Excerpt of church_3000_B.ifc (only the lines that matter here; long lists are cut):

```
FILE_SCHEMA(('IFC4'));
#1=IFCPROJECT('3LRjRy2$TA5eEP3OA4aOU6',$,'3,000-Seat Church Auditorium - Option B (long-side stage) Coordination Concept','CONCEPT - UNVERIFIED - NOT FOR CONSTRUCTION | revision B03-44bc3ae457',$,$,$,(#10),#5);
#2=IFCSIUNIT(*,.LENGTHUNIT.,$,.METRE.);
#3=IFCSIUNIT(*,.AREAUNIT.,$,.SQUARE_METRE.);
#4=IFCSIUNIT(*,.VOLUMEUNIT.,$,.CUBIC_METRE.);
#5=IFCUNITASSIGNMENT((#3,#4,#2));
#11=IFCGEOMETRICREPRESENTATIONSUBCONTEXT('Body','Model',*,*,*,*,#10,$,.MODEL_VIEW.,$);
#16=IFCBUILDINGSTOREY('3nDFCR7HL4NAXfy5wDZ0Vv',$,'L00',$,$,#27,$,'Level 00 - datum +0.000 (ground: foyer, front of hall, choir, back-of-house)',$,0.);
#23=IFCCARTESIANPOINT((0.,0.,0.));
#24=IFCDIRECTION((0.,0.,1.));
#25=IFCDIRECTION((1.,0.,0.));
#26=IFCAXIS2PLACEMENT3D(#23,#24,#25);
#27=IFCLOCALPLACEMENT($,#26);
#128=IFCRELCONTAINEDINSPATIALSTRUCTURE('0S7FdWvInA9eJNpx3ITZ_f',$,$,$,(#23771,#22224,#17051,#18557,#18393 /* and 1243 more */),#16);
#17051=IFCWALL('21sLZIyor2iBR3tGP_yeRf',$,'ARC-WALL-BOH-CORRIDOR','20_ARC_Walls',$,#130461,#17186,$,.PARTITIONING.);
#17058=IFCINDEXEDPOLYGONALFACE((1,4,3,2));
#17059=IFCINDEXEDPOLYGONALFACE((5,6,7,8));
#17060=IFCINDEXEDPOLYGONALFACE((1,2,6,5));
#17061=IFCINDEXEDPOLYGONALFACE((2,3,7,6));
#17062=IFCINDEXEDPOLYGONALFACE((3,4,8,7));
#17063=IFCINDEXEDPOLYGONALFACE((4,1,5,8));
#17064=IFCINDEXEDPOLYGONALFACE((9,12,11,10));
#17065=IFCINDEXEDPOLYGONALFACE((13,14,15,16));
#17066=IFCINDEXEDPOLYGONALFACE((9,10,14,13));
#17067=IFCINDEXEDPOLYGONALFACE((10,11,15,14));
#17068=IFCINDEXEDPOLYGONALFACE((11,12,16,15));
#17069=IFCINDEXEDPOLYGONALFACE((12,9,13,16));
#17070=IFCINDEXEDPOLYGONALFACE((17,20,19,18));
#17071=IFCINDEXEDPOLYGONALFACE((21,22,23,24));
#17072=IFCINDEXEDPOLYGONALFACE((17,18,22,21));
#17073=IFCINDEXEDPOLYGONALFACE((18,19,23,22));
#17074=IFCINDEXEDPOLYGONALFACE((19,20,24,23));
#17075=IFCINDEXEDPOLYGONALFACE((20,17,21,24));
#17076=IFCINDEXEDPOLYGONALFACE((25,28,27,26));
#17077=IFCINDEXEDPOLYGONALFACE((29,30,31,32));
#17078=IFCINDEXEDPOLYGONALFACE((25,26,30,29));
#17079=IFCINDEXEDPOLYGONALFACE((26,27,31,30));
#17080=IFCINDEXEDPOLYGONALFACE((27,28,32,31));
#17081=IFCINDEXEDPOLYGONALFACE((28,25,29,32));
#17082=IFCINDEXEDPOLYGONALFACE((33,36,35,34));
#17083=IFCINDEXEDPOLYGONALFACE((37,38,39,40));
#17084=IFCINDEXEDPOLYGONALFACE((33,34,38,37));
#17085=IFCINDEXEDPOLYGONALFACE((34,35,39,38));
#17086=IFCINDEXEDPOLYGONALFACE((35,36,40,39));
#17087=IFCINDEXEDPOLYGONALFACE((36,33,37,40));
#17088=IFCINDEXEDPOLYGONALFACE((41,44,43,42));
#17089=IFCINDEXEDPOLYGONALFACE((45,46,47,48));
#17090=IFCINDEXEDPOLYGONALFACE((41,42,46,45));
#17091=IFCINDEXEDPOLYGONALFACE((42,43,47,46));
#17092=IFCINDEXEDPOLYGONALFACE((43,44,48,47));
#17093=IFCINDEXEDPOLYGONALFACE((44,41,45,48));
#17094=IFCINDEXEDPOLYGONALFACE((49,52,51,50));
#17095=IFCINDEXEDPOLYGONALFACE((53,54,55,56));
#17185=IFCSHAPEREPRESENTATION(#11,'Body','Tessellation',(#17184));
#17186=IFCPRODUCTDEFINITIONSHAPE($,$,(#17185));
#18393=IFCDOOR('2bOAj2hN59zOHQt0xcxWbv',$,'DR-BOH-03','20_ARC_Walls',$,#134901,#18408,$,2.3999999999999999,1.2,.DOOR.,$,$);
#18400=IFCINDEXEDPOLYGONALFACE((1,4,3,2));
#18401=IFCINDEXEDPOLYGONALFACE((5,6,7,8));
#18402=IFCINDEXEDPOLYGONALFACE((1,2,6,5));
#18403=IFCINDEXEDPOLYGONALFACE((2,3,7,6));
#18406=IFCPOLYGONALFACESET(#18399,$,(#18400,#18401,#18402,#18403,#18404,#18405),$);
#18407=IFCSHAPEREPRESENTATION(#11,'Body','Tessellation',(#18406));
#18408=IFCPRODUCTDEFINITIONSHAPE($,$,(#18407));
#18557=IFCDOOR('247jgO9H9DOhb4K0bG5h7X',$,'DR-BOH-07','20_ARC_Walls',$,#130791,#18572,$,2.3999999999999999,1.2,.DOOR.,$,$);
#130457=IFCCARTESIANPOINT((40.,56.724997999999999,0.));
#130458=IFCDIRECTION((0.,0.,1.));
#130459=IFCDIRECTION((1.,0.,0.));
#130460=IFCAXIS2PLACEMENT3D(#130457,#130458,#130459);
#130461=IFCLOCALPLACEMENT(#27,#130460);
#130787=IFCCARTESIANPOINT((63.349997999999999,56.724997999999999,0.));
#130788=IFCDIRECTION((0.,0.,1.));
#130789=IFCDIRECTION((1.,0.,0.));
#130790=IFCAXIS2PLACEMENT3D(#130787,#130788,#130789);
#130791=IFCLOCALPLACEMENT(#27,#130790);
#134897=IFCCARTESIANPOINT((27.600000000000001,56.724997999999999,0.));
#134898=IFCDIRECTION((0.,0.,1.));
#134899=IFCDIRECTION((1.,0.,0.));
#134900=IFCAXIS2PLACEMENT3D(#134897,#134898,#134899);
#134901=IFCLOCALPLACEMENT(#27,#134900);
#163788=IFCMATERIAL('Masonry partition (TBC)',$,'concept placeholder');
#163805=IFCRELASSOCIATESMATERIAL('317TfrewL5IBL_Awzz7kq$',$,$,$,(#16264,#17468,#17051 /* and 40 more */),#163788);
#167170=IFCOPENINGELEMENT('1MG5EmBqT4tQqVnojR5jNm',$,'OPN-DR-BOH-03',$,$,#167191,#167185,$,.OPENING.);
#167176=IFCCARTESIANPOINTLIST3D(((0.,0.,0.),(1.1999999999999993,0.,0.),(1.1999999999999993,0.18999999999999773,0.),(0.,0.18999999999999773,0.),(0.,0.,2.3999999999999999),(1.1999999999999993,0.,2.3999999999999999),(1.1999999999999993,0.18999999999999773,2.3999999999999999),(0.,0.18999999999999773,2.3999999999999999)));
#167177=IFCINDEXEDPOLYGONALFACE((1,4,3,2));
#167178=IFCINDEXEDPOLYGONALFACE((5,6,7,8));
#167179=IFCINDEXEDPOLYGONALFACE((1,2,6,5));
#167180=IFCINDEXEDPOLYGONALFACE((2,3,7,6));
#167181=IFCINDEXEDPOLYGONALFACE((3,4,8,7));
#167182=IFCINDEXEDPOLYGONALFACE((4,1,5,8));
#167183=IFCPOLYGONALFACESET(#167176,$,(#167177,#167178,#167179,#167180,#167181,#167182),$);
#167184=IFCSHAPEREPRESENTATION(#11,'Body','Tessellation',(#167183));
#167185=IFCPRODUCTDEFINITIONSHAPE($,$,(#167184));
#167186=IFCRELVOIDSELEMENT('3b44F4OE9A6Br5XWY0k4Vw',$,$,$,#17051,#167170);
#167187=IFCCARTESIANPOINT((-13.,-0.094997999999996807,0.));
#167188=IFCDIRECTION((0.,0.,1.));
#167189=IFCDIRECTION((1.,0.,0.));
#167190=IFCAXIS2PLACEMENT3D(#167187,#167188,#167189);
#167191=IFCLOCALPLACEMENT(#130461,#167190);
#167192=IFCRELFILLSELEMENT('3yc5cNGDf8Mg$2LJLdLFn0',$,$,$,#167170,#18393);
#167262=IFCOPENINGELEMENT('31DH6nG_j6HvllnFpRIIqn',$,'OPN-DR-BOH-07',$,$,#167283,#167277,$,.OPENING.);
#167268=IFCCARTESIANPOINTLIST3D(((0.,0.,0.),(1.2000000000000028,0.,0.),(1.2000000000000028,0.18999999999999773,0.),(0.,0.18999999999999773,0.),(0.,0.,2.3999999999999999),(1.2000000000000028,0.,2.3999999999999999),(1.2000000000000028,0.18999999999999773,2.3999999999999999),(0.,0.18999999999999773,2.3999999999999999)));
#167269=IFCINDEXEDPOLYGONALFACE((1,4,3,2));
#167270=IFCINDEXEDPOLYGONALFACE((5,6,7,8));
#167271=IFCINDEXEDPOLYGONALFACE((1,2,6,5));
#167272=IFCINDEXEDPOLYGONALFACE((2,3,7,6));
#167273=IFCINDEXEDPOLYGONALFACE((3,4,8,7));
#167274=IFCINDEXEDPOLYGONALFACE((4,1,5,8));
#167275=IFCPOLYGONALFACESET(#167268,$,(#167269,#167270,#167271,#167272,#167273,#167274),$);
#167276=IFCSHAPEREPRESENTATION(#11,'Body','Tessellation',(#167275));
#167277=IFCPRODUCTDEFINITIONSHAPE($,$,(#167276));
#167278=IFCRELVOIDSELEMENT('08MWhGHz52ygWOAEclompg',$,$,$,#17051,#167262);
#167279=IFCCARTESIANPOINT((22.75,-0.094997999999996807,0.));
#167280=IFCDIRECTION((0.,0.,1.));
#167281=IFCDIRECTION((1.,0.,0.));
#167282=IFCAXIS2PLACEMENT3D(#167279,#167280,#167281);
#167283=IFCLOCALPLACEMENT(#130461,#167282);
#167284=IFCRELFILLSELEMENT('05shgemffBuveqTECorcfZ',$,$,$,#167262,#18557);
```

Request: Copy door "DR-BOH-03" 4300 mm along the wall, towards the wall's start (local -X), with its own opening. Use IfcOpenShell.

```python
import ifcopenshell
import ifcopenshell.api.feature
import ifcopenshell.api.geometry
import ifcopenshell.api.root
import ifcopenshell.geom
import ifcopenshell.util.element
import ifcopenshell.util.placement
import ifcopenshell.util.shape
import ifcopenshell.util.unit

model = ifcopenshell.open("church_3000_B.ifc")
unit_scale = ifcopenshell.util.unit.calculate_unit_scale(model)
settings = ifcopenshell.geom.settings()


def volume(element):
    """Net volume in cubic metres, openings subtracted."""
    shape = ifcopenshell.geom.create_shape(settings, element)
    return ifcopenshell.util.shape.get_volume(shape.geometry)


door = model.by_guid("2bOAj2hN59zOHQt0xcxWbv")
opening = door.FillsVoids[0].RelatingOpeningElement
wall = opening.VoidsElements[0].RelatingBuildingElement
before = volume(wall)
shift = ifcopenshell.util.placement.get_local_placement(wall.ObjectPlacement)[:3, 0] * -4.3 / unit_scale

# copy_class copies the void relationship, type, container and properties, but no geometry.
new_opening = ifcopenshell.api.root.copy_class(model, product=opening)
new_opening.Representation = ifcopenshell.util.element.copy_deep(
    model, opening.Representation, exclude=["IfcGeometricRepresentationContext", "IfcRepresentationMap"]
)
new_door = ifcopenshell.api.root.copy_class(model, product=door)
new_door.Representation = ifcopenshell.util.element.copy_deep(
    model, door.Representation, exclude=["IfcGeometricRepresentationContext", "IfcRepresentationMap"]
)
ifcopenshell.api.feature.add_filling(model, opening=new_opening, element=new_door)

for old, new in ((opening, new_opening), (door, new_door)):
    matrix = ifcopenshell.util.placement.get_local_placement(old.ObjectPlacement)
    matrix[:3, 3] += shift
    ifcopenshell.api.geometry.edit_object_placement(model, product=new, matrix=matrix, is_si=False)

after = volume(wall)

print(f"wall volume {before:.3f} -> {after:.3f} m3")

model.write("church_3000_B_updated.ifc")
```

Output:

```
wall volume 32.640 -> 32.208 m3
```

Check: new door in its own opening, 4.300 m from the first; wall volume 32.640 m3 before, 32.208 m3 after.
